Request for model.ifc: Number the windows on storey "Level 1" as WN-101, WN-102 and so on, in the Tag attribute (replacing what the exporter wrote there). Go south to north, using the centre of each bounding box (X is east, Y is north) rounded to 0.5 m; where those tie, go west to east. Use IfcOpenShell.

First a look at what the model holds.

```python
import ifcopenshell
import ifcopenshell.util.element
import ifcopenshell.util.placement

model = ifcopenshell.open("model.ifc")
print(model.schema)
storey = next(s for s in model.by_type("IfcBuildingStorey") if s.Name == "Level 1")
windows = [e for e in ifcopenshell.util.element.get_decomposition(storey) if e.is_a("IfcWindow")]
for e in sorted(windows, key=lambda e: e.id()):
    origin = ifcopenshell.util.placement.get_local_placement(e.ObjectPlacement)[:3, 3]
    print(e.id(), e.Tag, e.Name, origin.round(2) + 0.0, sep=" | ")
```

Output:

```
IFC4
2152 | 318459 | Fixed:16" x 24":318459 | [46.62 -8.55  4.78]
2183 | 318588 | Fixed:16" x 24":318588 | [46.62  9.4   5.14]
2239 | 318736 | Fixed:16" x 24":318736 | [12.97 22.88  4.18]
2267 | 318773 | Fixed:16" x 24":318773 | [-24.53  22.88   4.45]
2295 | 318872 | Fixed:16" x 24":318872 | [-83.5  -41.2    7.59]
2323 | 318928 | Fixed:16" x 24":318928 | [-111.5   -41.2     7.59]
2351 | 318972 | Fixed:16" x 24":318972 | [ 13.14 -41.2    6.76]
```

```python
import ifcopenshell
import ifcopenshell.geom
import ifcopenshell.util.element
import ifcopenshell.util.shape

model = ifcopenshell.open("model.ifc")
settings = ifcopenshell.geom.settings()
settings.set("use-world-coords", True)


def centre(element):
    shape = ifcopenshell.geom.create_shape(settings, element)
    return ifcopenshell.util.shape.get_bbox_centroid(shape.geometry)


storey = next(s for s in model.by_type("IfcBuildingStorey") if s.Name == "Level 1")
windows = [e for e in ifcopenshell.util.element.get_decomposition(storey) if e.is_a("IfcWindow")]

# Insertion points can sit at a corner or the storey origin, so sort by the geometry (in metres).
centres = {e: centre(e) for e in windows}
windows.sort(key=lambda e: (round(centres[e][1] / 0.5), centres[e][0]))

for i, e in enumerate(windows, start=1):
    number = f"WN-1{i:02d}"
    e.Tag = number
    print(e.id(), number)

model.write("model_v2.ifc")
```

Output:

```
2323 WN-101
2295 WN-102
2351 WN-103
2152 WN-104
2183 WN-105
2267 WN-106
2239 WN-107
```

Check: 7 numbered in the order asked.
